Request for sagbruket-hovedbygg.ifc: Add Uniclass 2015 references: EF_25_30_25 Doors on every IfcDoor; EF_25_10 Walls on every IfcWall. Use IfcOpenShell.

First a look at what the model holds.

```python
import ifcopenshell

model = ifcopenshell.open("sagbruket-hovedbygg.ifc")
print(model.schema)
print("classifications:", [c.Name for c in model.by_type("IfcClassification")])
for ifc_class in ("IfcDoor", "IfcRoof", "IfcStair", "IfcWall", "IfcWindow"):
    print(ifc_class, len(model.by_type(ifc_class)))
```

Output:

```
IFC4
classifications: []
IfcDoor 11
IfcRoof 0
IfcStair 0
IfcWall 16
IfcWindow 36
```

```python
import ifcopenshell
import ifcopenshell.api.classification

model = ifcopenshell.open("sagbruket-hovedbygg.ifc")

system = ifcopenshell.api.classification.add_classification(model, classification="Uniclass 2015")

codes = {
    "IfcDoor": ("EF_25_30_25", "Doors"),
    "IfcWall": ("EF_25_10", "Walls"),
}
for ifc_class, (code, name) in codes.items():
    products = model.by_type(ifc_class)
    ifcopenshell.api.classification.add_reference(
        model, products=products, classification=system, identification=code, name=name
    )
    print(code, len(products))

model.write("sagbruket-hovedbygg_v2.ifc")
```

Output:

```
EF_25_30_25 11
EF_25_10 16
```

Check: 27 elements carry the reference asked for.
